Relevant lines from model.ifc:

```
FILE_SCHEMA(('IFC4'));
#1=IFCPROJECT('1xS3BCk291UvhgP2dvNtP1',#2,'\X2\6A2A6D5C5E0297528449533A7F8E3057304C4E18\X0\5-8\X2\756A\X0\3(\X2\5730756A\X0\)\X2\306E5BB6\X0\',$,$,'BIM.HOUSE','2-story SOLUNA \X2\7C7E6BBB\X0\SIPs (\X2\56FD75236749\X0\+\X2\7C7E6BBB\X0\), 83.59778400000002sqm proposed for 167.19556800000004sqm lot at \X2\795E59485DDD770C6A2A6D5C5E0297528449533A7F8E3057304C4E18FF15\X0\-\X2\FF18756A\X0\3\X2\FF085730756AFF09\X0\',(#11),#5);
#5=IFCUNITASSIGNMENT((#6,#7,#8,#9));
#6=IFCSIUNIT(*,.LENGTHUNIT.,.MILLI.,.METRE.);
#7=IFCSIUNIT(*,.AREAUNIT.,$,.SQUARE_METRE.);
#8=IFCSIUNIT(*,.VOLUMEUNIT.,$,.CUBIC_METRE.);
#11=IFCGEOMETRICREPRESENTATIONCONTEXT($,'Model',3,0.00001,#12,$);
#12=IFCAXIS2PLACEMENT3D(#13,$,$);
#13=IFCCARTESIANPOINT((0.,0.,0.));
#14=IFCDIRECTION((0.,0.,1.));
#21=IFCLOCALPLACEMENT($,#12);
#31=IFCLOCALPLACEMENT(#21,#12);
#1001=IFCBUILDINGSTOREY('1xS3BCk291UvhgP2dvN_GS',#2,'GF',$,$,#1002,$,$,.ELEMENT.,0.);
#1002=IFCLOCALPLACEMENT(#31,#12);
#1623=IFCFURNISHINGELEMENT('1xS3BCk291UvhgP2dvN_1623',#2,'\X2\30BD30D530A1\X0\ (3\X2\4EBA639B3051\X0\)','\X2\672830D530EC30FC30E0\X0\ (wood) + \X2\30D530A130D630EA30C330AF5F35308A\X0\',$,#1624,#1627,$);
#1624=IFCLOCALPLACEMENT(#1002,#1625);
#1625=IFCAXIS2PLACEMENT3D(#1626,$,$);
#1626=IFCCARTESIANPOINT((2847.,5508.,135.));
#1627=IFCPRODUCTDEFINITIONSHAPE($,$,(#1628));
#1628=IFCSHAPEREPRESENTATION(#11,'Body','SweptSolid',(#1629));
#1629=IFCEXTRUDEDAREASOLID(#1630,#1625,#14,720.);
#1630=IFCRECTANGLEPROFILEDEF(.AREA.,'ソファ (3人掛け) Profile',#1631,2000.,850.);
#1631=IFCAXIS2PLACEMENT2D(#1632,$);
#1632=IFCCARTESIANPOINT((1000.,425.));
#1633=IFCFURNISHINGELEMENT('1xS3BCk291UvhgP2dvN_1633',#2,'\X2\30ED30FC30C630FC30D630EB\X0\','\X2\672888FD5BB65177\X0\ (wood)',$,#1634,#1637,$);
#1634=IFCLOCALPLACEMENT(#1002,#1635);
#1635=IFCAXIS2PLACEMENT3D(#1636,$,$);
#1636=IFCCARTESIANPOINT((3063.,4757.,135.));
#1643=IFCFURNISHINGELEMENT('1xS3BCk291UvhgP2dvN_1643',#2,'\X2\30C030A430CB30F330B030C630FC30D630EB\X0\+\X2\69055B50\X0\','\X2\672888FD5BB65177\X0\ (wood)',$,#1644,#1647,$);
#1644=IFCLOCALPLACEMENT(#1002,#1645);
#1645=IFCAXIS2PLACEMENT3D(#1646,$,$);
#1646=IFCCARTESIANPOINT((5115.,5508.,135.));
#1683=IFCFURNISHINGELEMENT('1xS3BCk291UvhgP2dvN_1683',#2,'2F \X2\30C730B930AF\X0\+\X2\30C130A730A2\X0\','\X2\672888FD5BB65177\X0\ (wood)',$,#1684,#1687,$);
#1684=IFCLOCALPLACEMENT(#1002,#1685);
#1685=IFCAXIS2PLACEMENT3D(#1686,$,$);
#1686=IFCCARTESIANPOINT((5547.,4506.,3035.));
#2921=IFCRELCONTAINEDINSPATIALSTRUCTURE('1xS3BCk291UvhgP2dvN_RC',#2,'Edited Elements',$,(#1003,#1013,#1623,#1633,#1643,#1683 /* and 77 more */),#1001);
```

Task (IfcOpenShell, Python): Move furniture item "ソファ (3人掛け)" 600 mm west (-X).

```python
import ifcopenshell
import ifcopenshell.api.geometry
import ifcopenshell.util.placement
import ifcopenshell.util.unit

model = ifcopenshell.open("model.ifc")
unit_scale = ifcopenshell.util.unit.calculate_unit_scale(model)

item = model.by_guid("1xS3BCk291UvhgP2dvN_1623")
matrix = ifcopenshell.util.placement.get_local_placement(item.ObjectPlacement)
matrix[0, 3] -= 0.6 / unit_scale
ifcopenshell.api.geometry.edit_object_placement(model, product=item, matrix=matrix, is_si=False)

print(ifcopenshell.util.placement.get_local_placement(item.ObjectPlacement).round(3) + 0.0)

model.write("model-out.ifc")
```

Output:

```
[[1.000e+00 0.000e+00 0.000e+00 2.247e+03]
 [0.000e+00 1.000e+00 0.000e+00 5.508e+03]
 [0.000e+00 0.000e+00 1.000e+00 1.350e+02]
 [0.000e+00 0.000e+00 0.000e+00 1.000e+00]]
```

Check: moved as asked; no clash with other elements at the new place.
